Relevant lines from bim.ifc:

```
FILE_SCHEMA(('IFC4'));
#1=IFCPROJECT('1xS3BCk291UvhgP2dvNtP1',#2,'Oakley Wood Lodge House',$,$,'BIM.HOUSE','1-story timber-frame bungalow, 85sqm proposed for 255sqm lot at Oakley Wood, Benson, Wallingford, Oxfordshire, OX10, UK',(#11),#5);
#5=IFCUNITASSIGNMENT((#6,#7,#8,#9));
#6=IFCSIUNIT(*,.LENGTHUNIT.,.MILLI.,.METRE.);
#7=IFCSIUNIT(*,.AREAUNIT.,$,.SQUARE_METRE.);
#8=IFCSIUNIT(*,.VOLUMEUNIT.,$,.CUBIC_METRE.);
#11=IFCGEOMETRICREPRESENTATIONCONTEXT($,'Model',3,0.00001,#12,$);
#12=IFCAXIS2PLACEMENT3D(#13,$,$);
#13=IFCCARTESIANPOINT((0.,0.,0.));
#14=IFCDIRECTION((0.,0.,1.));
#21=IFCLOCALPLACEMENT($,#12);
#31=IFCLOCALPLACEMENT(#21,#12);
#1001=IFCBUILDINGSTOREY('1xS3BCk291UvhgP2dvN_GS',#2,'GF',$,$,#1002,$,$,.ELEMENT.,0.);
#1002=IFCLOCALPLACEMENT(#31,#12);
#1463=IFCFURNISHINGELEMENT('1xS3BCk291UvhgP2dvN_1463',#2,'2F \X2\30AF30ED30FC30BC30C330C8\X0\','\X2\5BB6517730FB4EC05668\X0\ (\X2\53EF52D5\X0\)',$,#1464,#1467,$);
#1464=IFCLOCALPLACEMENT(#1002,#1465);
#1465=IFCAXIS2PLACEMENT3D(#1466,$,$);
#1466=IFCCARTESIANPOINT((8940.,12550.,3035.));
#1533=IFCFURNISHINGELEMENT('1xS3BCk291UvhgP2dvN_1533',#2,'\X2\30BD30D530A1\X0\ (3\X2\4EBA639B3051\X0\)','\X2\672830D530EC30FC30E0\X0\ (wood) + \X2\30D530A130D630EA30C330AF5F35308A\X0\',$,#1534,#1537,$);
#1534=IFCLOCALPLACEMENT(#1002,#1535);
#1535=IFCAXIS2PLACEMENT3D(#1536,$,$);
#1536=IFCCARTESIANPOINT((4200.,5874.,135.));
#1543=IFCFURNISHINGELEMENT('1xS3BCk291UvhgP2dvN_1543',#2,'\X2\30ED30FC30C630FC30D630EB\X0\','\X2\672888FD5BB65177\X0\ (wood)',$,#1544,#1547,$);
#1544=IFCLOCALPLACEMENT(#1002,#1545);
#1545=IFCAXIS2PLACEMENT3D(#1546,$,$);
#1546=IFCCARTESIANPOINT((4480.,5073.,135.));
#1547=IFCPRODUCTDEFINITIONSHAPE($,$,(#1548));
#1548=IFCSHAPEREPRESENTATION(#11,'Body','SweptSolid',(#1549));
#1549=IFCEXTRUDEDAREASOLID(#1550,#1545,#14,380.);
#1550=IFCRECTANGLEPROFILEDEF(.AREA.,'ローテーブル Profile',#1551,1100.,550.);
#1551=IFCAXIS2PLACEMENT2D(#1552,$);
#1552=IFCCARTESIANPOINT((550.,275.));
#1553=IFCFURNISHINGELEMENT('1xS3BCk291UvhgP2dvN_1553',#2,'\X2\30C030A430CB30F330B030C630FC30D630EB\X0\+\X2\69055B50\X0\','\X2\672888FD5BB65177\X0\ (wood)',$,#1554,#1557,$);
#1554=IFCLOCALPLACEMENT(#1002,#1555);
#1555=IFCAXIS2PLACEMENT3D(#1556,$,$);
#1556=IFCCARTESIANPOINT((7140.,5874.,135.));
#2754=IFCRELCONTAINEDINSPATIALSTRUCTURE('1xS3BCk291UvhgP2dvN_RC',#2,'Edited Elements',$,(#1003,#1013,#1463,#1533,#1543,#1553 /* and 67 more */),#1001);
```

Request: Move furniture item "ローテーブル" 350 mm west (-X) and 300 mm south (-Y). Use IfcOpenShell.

```python
import ifcopenshell
import ifcopenshell.api.geometry
import ifcopenshell.util.placement
import ifcopenshell.util.unit

model = ifcopenshell.open("bim.ifc")
unit_scale = ifcopenshell.util.unit.calculate_unit_scale(model)

item = model.by_guid("1xS3BCk291UvhgP2dvN_1543")
matrix = ifcopenshell.util.placement.get_local_placement(item.ObjectPlacement)
matrix[0, 3] -= 0.35 / unit_scale
matrix[1, 3] -= 0.3 / unit_scale
ifcopenshell.api.geometry.edit_object_placement(model, product=item, matrix=matrix, is_si=False)

print(ifcopenshell.util.placement.get_local_placement(item.ObjectPlacement).round(3) + 0.0)

model.write("bim_edited.ifc")
```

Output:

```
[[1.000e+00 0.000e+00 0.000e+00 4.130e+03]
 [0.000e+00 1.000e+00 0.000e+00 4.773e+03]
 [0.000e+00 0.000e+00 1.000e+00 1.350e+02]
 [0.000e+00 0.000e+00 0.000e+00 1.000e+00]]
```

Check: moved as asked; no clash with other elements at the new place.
